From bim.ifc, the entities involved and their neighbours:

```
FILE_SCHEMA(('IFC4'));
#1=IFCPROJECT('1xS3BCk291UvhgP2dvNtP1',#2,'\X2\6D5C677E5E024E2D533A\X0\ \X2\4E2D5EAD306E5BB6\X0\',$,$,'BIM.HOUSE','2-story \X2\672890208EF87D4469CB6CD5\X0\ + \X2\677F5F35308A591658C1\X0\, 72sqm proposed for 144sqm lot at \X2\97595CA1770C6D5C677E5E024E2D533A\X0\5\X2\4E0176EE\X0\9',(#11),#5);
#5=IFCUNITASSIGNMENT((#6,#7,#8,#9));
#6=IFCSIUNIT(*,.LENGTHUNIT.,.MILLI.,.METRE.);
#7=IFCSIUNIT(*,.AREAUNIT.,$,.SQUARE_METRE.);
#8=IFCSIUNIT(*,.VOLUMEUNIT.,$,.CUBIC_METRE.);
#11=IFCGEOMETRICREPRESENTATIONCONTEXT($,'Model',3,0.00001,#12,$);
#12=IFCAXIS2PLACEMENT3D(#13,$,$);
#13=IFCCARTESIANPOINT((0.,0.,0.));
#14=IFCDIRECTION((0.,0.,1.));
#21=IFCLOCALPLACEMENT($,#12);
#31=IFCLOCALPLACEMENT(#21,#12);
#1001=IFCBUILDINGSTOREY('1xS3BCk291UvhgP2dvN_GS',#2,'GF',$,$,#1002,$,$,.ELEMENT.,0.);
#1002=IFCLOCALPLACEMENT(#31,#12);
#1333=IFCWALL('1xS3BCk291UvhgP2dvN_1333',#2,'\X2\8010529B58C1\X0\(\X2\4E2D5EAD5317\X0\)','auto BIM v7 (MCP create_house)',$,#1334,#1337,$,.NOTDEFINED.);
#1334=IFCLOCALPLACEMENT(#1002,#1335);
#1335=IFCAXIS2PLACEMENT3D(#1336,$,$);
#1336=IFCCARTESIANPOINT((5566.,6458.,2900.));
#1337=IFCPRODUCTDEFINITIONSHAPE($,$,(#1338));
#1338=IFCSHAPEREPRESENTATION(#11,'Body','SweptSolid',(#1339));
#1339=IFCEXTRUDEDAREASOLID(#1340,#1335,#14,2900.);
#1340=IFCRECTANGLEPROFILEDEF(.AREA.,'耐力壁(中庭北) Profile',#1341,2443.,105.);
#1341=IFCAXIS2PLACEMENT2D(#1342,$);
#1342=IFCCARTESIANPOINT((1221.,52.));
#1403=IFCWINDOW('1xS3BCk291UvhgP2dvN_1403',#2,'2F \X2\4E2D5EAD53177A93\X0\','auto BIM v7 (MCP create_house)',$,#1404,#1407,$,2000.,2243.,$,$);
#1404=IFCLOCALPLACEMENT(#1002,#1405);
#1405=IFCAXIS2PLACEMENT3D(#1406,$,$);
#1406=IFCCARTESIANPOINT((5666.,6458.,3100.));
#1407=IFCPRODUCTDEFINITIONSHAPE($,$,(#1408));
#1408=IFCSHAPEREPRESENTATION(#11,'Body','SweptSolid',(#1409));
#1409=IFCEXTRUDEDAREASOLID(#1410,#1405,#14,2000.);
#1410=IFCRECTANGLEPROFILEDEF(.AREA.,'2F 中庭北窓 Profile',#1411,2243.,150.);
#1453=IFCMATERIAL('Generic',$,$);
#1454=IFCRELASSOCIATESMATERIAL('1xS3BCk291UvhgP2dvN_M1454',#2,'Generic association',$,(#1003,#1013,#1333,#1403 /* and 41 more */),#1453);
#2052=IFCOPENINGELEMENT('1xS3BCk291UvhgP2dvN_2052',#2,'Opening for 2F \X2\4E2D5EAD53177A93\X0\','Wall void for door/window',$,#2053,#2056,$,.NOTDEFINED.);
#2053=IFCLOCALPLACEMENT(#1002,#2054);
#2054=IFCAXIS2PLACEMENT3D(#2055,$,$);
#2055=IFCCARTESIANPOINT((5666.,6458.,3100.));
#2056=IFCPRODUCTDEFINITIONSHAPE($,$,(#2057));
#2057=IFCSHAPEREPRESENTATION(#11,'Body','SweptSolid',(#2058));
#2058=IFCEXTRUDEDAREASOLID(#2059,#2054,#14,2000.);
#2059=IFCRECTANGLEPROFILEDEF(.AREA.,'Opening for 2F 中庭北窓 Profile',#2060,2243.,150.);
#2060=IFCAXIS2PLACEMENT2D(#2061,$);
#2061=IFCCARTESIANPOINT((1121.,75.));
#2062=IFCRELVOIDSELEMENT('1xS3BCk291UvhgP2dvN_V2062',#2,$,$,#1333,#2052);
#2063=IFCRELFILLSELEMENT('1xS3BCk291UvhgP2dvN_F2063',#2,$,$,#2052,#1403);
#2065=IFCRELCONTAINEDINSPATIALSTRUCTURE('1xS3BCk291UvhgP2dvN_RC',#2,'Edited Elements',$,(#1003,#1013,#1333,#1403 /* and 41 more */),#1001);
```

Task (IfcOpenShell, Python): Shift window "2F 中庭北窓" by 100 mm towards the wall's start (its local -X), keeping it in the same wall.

```python
import ifcopenshell
import ifcopenshell.api.geometry
import ifcopenshell.util.placement

model = ifcopenshell.open("bim.ifc")

window = model.by_guid("1xS3BCk291UvhgP2dvN_1403")
opening = window.FillsVoids[0].RelatingOpeningElement
wall = opening.VoidsElements[0].RelatingBuildingElement

wall_matrix = ifcopenshell.util.placement.get_local_placement(wall.ObjectPlacement)
shift = wall_matrix[:3, 0] * -100.0
before = ifcopenshell.util.placement.get_local_placement(window.ObjectPlacement)[:3, 3].copy()

# The window is not placed relative to its opening, so move both.
for product in (opening, window):
    matrix = ifcopenshell.util.placement.get_local_placement(product.ObjectPlacement)
    matrix[:3, 3] += shift
    ifcopenshell.api.geometry.edit_object_placement(model, product=product, matrix=matrix, is_si=False)

after = ifcopenshell.util.placement.get_local_placement(window.ObjectPlacement)[:3, 3]
print("window moved by", (after - before).round(3) + 0.0)

model.write("bim_updated.ifc")
```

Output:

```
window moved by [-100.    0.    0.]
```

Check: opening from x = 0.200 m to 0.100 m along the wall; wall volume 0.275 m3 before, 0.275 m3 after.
